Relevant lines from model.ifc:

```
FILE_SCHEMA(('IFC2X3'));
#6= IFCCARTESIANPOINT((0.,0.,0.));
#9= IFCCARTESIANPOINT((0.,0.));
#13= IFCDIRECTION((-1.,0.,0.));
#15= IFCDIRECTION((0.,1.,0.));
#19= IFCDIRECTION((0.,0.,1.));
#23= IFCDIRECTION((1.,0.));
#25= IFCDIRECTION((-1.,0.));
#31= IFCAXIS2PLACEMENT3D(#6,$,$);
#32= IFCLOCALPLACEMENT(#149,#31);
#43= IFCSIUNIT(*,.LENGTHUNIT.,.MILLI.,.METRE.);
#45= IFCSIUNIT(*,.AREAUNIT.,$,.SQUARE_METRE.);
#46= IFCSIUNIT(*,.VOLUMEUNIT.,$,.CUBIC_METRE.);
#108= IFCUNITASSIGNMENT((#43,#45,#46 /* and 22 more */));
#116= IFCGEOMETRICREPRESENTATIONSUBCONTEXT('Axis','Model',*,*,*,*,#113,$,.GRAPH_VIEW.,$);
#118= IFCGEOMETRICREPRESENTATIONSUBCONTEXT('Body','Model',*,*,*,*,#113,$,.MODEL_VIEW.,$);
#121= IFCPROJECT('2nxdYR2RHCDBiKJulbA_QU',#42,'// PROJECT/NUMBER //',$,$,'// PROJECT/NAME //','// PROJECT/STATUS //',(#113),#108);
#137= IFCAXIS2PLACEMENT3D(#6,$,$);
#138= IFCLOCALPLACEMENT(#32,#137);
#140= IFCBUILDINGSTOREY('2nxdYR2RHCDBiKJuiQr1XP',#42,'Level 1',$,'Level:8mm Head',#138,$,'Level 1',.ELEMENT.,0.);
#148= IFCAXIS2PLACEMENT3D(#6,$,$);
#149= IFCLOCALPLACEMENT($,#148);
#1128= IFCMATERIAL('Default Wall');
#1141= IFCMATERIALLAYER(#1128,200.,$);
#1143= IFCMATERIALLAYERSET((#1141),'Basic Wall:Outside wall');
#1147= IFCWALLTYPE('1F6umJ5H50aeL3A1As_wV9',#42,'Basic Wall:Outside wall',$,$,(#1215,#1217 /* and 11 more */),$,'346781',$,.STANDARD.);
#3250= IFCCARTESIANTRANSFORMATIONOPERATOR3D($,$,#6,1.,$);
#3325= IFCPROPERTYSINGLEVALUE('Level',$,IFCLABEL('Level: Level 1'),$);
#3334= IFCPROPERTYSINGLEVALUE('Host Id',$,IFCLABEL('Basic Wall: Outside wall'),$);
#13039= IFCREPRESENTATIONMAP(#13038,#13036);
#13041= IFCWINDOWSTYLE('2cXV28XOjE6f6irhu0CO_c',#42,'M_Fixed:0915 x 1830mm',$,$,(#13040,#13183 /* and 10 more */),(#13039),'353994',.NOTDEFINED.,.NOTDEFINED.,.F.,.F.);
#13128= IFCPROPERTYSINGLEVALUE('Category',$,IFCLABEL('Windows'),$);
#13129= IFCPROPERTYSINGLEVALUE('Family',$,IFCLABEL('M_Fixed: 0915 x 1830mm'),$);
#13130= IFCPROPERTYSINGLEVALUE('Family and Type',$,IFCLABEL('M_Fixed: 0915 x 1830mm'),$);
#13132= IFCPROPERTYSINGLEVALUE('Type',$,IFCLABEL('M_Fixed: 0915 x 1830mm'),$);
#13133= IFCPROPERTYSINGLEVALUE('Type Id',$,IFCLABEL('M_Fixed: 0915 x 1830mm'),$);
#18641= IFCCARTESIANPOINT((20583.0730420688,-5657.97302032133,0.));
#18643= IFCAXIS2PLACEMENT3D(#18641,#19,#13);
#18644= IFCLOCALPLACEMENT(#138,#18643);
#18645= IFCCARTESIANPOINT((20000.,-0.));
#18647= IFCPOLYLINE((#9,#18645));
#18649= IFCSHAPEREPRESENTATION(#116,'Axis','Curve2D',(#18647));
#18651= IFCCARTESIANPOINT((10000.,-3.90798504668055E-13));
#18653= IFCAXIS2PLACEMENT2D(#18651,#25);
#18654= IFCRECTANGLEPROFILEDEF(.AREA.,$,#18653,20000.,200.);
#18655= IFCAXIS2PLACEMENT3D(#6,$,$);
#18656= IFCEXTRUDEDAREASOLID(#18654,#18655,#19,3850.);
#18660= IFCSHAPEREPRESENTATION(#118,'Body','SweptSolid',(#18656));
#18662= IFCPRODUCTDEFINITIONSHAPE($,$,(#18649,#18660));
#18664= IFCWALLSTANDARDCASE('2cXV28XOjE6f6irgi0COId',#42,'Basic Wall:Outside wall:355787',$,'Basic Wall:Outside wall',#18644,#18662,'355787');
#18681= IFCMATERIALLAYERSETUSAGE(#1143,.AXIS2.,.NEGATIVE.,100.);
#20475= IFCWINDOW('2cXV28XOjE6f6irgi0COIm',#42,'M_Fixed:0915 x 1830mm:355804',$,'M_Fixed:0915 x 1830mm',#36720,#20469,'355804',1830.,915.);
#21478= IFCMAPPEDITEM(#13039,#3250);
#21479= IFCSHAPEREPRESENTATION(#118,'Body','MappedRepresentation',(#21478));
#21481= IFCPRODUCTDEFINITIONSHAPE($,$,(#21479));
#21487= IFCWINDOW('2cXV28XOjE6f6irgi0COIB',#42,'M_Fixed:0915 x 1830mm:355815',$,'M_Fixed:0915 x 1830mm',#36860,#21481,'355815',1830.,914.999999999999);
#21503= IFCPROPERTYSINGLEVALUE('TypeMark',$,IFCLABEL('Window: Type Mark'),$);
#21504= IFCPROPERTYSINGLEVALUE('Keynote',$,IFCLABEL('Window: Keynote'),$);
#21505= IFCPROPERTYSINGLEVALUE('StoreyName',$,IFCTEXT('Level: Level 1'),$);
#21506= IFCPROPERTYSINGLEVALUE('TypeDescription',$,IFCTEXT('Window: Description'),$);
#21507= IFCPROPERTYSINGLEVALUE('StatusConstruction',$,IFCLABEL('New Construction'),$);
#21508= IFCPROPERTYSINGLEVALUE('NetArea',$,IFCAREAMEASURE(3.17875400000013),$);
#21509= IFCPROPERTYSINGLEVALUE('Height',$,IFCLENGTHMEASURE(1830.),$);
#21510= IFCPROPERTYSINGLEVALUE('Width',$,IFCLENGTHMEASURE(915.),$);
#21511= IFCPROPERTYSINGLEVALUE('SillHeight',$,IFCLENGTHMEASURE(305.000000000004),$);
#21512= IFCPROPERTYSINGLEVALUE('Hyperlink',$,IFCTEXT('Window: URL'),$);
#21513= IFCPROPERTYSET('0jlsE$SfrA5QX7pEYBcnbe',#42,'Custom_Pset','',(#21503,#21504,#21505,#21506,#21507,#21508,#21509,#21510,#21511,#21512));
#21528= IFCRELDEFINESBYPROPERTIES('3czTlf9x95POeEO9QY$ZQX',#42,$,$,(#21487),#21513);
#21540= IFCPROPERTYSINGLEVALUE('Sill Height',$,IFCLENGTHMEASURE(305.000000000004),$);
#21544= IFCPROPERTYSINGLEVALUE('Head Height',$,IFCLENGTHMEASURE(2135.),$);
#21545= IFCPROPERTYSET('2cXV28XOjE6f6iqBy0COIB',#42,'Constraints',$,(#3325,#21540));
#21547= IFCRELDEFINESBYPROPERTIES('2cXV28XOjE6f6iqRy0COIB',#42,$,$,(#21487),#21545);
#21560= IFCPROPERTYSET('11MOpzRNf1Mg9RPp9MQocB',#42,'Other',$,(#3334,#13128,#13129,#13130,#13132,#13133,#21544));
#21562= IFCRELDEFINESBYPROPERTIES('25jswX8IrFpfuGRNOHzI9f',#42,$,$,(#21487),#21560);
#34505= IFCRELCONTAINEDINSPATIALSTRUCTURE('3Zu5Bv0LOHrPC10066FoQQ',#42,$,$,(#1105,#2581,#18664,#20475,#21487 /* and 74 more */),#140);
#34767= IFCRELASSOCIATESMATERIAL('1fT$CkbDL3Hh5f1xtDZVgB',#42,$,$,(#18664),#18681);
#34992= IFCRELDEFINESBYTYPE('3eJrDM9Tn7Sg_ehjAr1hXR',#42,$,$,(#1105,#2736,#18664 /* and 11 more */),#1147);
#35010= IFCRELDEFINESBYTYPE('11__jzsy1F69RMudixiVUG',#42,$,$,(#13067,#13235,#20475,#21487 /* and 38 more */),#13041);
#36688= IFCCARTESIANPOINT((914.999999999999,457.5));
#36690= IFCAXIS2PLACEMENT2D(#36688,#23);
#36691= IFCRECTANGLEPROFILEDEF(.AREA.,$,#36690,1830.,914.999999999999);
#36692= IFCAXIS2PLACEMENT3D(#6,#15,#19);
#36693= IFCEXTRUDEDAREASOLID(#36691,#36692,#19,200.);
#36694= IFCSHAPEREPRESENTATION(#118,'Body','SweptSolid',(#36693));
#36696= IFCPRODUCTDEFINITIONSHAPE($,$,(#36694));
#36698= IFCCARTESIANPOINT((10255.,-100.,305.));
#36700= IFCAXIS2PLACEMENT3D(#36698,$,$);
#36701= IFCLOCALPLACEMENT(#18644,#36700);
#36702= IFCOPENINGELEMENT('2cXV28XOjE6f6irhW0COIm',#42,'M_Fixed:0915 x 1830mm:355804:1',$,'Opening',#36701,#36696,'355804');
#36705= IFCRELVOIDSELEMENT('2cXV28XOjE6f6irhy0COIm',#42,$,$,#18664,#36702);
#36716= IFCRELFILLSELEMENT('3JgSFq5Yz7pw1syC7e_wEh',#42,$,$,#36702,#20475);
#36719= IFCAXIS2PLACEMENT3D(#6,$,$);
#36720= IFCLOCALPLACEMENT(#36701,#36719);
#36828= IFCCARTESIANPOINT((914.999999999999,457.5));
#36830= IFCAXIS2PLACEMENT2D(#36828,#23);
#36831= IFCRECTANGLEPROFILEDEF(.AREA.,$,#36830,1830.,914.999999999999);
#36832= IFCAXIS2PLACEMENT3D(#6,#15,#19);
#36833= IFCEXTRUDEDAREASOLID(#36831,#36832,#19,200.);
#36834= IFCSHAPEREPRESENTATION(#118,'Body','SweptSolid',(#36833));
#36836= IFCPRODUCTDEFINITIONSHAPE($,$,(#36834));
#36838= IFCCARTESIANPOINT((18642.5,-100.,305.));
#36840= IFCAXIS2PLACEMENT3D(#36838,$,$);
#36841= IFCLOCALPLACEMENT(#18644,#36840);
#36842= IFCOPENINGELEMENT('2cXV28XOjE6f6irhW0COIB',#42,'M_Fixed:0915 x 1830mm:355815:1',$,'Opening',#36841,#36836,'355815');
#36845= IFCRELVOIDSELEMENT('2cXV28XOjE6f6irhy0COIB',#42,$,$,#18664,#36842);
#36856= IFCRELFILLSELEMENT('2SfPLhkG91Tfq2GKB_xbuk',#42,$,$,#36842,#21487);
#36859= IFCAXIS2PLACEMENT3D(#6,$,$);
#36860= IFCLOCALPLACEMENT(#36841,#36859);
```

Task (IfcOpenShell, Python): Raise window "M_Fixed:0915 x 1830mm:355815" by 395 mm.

```python
import numpy as np
import ifcopenshell
import ifcopenshell.api.geometry
import ifcopenshell.api.pset
import ifcopenshell.util.element
import ifcopenshell.util.placement
import ifcopenshell.util.unit

model = ifcopenshell.open("model.ifc")
unit_scale = ifcopenshell.util.unit.calculate_unit_scale(model)

window = model.by_guid("2cXV28XOjE6f6irgi0COIB")
opening = window.FillsVoids[0].RelatingOpeningElement
dz = 0.395 / unit_scale

shift = np.array([0.0, 0.0, dz])
# The window is placed relative to its opening, so it follows when the opening moves.
matrix = ifcopenshell.util.placement.get_local_placement(opening.ObjectPlacement)
matrix[:3, 3] += shift
ifcopenshell.api.geometry.edit_object_placement(
    model, product=opening, matrix=matrix, is_si=False, should_transform_children=True
)

# Keep the stored heights in step.
pset = model.by_id(ifcopenshell.util.element.get_pset(window, "Custom_Pset", should_inherit=False)["id"])
ifcopenshell.api.pset.edit_pset(model, pset=pset, properties={
    "SillHeight": model.create_entity("IfcLengthMeasure", ifcopenshell.util.element.get_pset(window, "Constraints", "Sill Height") + dz),
})
pset = model.by_id(ifcopenshell.util.element.get_pset(window, "Constraints", should_inherit=False)["id"])
ifcopenshell.api.pset.edit_pset(model, pset=pset, properties={
    "Sill Height": model.create_entity("IfcLengthMeasure", ifcopenshell.util.element.get_pset(window, "Constraints", "Sill Height") + dz),
})
pset = model.by_id(ifcopenshell.util.element.get_pset(window, "Other", should_inherit=False)["id"])
ifcopenshell.api.pset.edit_pset(model, pset=pset, properties={
    "Head Height": model.create_entity("IfcLengthMeasure", ifcopenshell.util.element.get_pset(window, "Other", "Head Height") + dz),
})

print(f"moved by {dz * unit_scale:+.3f} m")

model.write("model_edited.ifc")
```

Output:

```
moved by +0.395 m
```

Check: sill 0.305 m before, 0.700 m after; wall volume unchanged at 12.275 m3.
